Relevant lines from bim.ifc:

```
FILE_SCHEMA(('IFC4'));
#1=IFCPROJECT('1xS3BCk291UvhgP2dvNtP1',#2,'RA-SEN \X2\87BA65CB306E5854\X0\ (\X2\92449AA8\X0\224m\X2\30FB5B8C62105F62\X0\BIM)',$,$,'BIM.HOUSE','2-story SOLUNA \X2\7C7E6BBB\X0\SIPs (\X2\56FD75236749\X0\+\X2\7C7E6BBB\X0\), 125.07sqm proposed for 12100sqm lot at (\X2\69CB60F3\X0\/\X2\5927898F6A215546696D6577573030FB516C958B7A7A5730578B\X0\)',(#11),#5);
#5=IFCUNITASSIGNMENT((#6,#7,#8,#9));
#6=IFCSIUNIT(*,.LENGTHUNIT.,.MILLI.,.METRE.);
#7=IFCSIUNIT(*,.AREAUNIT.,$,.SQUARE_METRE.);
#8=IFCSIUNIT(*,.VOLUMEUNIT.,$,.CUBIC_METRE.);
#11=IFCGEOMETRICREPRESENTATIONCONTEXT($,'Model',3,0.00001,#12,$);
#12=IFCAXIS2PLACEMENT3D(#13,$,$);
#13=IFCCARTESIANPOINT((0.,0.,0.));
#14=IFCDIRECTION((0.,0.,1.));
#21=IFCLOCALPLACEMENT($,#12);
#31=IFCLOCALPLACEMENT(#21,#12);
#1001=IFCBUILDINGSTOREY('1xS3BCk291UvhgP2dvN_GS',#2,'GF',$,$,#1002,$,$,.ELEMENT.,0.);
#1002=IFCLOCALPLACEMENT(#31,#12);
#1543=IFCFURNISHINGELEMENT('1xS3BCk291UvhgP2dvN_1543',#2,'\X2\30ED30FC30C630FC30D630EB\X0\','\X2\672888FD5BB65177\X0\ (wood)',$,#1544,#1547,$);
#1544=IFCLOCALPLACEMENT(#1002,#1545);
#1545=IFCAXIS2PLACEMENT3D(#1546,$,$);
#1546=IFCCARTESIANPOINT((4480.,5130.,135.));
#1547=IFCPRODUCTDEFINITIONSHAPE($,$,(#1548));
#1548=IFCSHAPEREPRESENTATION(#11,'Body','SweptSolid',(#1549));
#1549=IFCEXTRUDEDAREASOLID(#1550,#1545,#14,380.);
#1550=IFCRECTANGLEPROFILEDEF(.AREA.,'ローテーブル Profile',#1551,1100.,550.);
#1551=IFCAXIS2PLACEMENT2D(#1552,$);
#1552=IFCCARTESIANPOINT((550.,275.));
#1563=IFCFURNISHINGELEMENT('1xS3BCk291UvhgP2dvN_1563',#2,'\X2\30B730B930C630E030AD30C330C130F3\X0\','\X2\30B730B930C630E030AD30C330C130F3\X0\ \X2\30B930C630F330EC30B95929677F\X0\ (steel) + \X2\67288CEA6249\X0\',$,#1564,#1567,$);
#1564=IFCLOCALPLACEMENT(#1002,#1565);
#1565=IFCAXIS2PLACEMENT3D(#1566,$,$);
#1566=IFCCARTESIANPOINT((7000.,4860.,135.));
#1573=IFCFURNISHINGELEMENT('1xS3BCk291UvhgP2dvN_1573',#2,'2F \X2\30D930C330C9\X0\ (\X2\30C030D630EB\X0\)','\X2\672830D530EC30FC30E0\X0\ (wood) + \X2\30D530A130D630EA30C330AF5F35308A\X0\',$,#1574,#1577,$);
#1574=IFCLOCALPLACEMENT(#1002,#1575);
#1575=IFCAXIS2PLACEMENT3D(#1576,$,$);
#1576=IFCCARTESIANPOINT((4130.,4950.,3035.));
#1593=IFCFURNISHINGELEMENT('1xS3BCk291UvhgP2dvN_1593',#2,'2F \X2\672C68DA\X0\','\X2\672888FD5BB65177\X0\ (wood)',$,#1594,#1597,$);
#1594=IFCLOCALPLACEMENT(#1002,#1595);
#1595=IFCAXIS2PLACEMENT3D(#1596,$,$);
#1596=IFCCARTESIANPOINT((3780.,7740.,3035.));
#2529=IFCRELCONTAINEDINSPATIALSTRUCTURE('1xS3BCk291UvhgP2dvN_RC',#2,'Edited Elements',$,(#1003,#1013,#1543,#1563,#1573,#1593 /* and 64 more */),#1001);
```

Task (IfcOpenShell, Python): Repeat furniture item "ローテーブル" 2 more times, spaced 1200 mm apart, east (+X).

```python
import numpy as np
import ifcopenshell
import ifcopenshell.api.geometry
import ifcopenshell.api.root
import ifcopenshell.util.element
import ifcopenshell.util.placement

model = ifcopenshell.open("bim.ifc")


def reuse_history(source, copy):
    """copy_class also copies each property set's owner history, people and application; keep the originals."""
    for rel in copy.IsDefinedBy:
        if rel.is_a("IfcRelDefinesByProperties") and (history := rel.RelatingPropertyDefinition.OwnerHistory):
            rel.RelatingPropertyDefinition.OwnerHistory = source.OwnerHistory
            ifcopenshell.util.element.remove_deep2(model, history)


source = model.by_id(1543)
base = ifcopenshell.util.placement.get_local_placement(source.ObjectPlacement)
step = np.array([1.0, 0.0, 0.0]) * 1200.0

for i in range(1, 3):
    copy = ifcopenshell.api.root.copy_class(model, product=source)
    copy.Representation = ifcopenshell.util.element.copy_deep(
        model, source.Representation, exclude=["IfcGeometricRepresentationContext", "IfcRepresentationMap"]
    )
    reuse_history(source, copy)
    matrix = base.copy()
    matrix[:3, 3] += i * step
    print("added at", matrix[:3, 3].round(3) + 0.0)
    ifcopenshell.api.geometry.edit_object_placement(model, product=copy, matrix=matrix, is_si=False)

model.write("bim_edited.ifc")
```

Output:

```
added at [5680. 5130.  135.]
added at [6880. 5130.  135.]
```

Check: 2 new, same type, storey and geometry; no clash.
